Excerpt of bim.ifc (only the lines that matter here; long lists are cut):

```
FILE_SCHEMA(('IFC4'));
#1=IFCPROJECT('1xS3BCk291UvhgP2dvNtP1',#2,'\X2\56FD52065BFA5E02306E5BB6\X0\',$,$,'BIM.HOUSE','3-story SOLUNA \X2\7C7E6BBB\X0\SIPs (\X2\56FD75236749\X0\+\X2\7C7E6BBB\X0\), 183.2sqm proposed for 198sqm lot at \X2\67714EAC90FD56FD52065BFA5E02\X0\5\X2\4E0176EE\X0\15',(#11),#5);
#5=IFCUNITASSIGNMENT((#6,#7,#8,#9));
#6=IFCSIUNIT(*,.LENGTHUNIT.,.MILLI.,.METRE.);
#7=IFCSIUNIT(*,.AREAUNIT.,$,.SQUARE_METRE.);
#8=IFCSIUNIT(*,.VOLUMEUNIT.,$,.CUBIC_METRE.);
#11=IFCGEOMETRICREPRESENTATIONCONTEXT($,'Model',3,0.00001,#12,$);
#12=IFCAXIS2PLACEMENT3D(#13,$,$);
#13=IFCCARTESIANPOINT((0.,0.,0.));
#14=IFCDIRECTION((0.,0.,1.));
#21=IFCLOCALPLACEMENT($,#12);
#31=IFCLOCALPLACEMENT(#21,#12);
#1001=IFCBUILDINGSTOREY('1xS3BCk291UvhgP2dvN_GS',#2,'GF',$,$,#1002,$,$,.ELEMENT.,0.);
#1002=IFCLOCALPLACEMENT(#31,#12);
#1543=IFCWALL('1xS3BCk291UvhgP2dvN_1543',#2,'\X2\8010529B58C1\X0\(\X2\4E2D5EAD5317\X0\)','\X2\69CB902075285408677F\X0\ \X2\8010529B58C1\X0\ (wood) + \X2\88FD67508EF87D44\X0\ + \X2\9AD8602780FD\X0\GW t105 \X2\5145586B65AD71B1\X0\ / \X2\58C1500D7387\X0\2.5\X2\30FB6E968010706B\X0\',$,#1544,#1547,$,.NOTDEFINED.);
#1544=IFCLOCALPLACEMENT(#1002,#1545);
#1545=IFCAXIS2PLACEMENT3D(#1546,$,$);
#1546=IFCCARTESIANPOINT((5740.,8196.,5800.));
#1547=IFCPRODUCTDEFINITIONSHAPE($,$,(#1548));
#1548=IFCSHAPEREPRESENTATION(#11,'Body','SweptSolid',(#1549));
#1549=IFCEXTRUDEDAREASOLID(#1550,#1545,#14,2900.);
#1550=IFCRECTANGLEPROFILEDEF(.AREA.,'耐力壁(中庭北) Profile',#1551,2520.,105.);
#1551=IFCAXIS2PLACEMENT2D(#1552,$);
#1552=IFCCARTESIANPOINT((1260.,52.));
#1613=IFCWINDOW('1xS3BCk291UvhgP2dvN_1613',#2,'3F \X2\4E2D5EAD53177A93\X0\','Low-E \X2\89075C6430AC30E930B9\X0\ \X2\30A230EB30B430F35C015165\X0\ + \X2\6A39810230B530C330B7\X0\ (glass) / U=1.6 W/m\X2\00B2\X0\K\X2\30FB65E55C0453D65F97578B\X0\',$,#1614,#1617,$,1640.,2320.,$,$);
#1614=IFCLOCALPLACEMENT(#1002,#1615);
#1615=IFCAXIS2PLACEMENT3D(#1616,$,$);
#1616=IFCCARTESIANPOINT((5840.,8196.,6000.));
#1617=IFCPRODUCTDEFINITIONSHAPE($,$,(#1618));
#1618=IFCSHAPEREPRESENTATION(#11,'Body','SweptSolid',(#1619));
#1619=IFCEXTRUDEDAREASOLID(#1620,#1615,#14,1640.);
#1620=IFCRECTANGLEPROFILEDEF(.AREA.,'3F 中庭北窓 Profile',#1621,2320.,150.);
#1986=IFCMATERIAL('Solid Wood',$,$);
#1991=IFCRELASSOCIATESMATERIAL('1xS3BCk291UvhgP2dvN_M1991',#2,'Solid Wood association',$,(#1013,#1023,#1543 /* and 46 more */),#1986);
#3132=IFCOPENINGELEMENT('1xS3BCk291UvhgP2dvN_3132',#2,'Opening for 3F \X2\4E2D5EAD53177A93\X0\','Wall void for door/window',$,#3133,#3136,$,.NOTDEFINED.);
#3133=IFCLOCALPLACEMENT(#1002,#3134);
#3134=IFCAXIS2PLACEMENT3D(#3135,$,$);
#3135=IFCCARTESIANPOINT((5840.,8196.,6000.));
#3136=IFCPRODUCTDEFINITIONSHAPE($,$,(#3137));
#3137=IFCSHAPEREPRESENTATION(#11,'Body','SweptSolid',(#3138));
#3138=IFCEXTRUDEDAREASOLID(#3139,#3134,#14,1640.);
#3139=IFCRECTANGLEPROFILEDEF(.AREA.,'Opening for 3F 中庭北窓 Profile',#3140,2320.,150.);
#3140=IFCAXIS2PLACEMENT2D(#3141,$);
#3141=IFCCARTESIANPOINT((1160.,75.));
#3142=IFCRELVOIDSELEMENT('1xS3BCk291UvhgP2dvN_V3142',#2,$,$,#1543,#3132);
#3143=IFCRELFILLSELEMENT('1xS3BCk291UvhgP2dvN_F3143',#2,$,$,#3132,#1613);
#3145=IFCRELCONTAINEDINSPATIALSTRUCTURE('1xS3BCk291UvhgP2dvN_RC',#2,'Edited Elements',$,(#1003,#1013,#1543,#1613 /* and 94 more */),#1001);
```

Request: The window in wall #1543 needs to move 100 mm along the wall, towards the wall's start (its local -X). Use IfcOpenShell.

```python
import ifcopenshell
import ifcopenshell.api.geometry
import ifcopenshell.util.placement

model = ifcopenshell.open("bim.ifc")

window = model.by_guid("1xS3BCk291UvhgP2dvN_1613")
opening = window.FillsVoids[0].RelatingOpeningElement
wall = opening.VoidsElements[0].RelatingBuildingElement

wall_matrix = ifcopenshell.util.placement.get_local_placement(wall.ObjectPlacement)
shift = wall_matrix[:3, 0] * -100.0
before = ifcopenshell.util.placement.get_local_placement(window.ObjectPlacement)[:3, 3].copy()

# The window is not placed relative to its opening, so move both.
for product in (opening, window):
    matrix = ifcopenshell.util.placement.get_local_placement(product.ObjectPlacement)
    matrix[:3, 3] += shift
    ifcopenshell.api.geometry.edit_object_placement(model, product=product, matrix=matrix, is_si=False)

after = ifcopenshell.util.placement.get_local_placement(window.ObjectPlacement)[:3, 3]
print("window moved by", (after - before).round(3) + 0.0)

model.write("bim_v2.ifc")
```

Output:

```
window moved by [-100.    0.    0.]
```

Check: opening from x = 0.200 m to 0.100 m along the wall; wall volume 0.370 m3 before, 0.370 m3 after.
